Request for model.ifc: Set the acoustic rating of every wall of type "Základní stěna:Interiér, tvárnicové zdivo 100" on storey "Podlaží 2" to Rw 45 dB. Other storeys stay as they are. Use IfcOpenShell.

First a look at what the model holds.

```python
import ifcopenshell
import ifcopenshell.util.element

model = ifcopenshell.open("model.ifc")
print(model.schema)
storey = next(s for s in model.by_type("IfcBuildingStorey") if s.Name == "Podlaží 2")
walls = [e for e in ifcopenshell.util.element.get_decomposition(storey) if e.is_a("IfcWall")]
seen = {}
for e in walls:
    element_type = ifcopenshell.util.element.get_type(e)
    key = (element_type.Name if element_type != e and element_type else None, ifcopenshell.util.element.get_pset(e, "Pset_WallCommon", "AcousticRating"))
    seen[key] = seen.get(key, 0) + 1
for (name, value), count in sorted(seen.items(), key=str):
    print(count, "x", name, "|", value)
```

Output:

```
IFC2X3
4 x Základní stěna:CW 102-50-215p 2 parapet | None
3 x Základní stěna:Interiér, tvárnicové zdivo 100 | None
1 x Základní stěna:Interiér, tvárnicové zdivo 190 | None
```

```python
import ifcopenshell
import ifcopenshell.api.pset
import ifcopenshell.util.element

model = ifcopenshell.open("model.ifc")

storey = next(s for s in model.by_type("IfcBuildingStorey") if s.Name == "Podlaží 2")
walls = [e for e in ifcopenshell.util.element.get_decomposition(storey) if e.is_a("IfcWall")]

count = 0
for e in walls:
    element_type = ifcopenshell.util.element.get_type(e)
    if element_type in (None, e) or element_type.Name != "Základní stěna:Interiér, tvárnicové zdivo 100":
        continue
    # add_pset returns the element's existing set when there is one.
    pset = ifcopenshell.api.pset.add_pset(model, product=e, name="Pset_WallCommon")
    ifcopenshell.api.pset.edit_pset(model, pset=pset, properties={"AcousticRating": "Rw 45 dB"})
    count += 1

print(count, "walls updated")

model.write("model_edited.ifc")
```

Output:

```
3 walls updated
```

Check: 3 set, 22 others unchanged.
